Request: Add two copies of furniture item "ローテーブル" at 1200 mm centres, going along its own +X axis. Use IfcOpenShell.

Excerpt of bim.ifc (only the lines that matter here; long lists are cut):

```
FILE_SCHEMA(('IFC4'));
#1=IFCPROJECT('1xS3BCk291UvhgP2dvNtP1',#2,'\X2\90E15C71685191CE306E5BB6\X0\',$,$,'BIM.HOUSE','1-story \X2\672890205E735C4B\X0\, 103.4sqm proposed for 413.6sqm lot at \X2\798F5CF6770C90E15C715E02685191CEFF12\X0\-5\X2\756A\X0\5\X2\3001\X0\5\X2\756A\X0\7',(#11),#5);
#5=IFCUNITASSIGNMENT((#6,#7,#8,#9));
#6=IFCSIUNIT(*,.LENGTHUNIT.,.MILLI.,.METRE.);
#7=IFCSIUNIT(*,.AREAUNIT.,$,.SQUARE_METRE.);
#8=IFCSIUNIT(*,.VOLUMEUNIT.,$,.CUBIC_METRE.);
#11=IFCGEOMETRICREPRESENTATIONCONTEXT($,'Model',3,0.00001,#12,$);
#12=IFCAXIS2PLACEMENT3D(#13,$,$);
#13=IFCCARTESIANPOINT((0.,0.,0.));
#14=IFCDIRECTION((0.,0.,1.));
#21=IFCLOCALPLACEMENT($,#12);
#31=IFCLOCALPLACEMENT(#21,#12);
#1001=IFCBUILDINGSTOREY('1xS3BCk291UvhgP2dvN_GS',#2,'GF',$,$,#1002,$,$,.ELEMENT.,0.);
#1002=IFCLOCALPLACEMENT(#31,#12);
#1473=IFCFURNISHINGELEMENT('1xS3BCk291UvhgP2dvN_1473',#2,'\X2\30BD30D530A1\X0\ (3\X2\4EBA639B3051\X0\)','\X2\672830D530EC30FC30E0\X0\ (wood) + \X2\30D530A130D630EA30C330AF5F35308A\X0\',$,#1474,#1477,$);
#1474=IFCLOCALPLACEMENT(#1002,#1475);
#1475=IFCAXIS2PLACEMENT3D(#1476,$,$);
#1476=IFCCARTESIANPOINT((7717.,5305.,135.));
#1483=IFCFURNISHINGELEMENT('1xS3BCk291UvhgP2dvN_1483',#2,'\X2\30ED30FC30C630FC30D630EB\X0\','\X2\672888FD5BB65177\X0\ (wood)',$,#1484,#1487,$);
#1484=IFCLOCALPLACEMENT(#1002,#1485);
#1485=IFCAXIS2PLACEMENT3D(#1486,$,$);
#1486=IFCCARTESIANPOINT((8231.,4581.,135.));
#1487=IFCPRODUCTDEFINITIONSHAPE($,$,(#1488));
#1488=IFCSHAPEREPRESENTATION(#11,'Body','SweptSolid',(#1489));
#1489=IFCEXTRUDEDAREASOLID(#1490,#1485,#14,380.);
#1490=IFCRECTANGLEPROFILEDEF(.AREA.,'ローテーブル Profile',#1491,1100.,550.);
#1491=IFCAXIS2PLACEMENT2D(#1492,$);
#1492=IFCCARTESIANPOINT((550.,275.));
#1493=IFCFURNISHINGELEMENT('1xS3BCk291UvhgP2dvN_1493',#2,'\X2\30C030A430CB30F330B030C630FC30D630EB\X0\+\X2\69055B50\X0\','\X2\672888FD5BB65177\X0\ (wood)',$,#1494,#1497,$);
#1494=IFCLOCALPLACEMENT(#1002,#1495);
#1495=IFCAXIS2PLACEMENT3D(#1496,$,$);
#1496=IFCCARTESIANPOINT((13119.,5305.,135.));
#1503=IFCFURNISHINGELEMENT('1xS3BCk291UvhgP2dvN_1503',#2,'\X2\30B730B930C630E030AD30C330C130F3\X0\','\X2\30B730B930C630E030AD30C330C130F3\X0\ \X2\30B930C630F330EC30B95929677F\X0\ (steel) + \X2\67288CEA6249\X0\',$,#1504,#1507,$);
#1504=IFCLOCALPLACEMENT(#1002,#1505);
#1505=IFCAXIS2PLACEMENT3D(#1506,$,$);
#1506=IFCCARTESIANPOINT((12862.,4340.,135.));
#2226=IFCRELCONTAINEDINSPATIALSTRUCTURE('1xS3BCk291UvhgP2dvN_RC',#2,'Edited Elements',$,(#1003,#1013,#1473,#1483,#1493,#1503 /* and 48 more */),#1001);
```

```python
import ifcopenshell
import ifcopenshell.api.geometry
import ifcopenshell.api.root
import ifcopenshell.util.element
import ifcopenshell.util.placement
import ifcopenshell.util.unit

model = ifcopenshell.open("bim.ifc")
unit_scale = ifcopenshell.util.unit.calculate_unit_scale(model)


def reuse_history(source, copy):
    """copy_class also copies each property set's owner history, people and application; keep the originals."""
    for rel in copy.IsDefinedBy:
        if rel.is_a("IfcRelDefinesByProperties") and (history := rel.RelatingPropertyDefinition.OwnerHistory):
            rel.RelatingPropertyDefinition.OwnerHistory = source.OwnerHistory
            ifcopenshell.util.element.remove_deep2(model, history)


source = model.by_guid("1xS3BCk291UvhgP2dvN_1483")
base = ifcopenshell.util.placement.get_local_placement(source.ObjectPlacement)
step = base[:3, 0] * 1.2 / unit_scale

for i in range(1, 3):
    copy = ifcopenshell.api.root.copy_class(model, product=source)
    copy.Representation = ifcopenshell.util.element.copy_deep(
        model, source.Representation, exclude=["IfcGeometricRepresentationContext", "IfcRepresentationMap"]
    )
    reuse_history(source, copy)
    matrix = base.copy()
    matrix[:3, 3] += i * step
    print("added at", matrix[:3, 3].round(3) + 0.0)
    ifcopenshell.api.geometry.edit_object_placement(model, product=copy, matrix=matrix, is_si=False)

model.write("bim_edited.ifc")
```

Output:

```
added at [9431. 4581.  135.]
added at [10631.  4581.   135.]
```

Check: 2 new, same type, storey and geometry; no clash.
